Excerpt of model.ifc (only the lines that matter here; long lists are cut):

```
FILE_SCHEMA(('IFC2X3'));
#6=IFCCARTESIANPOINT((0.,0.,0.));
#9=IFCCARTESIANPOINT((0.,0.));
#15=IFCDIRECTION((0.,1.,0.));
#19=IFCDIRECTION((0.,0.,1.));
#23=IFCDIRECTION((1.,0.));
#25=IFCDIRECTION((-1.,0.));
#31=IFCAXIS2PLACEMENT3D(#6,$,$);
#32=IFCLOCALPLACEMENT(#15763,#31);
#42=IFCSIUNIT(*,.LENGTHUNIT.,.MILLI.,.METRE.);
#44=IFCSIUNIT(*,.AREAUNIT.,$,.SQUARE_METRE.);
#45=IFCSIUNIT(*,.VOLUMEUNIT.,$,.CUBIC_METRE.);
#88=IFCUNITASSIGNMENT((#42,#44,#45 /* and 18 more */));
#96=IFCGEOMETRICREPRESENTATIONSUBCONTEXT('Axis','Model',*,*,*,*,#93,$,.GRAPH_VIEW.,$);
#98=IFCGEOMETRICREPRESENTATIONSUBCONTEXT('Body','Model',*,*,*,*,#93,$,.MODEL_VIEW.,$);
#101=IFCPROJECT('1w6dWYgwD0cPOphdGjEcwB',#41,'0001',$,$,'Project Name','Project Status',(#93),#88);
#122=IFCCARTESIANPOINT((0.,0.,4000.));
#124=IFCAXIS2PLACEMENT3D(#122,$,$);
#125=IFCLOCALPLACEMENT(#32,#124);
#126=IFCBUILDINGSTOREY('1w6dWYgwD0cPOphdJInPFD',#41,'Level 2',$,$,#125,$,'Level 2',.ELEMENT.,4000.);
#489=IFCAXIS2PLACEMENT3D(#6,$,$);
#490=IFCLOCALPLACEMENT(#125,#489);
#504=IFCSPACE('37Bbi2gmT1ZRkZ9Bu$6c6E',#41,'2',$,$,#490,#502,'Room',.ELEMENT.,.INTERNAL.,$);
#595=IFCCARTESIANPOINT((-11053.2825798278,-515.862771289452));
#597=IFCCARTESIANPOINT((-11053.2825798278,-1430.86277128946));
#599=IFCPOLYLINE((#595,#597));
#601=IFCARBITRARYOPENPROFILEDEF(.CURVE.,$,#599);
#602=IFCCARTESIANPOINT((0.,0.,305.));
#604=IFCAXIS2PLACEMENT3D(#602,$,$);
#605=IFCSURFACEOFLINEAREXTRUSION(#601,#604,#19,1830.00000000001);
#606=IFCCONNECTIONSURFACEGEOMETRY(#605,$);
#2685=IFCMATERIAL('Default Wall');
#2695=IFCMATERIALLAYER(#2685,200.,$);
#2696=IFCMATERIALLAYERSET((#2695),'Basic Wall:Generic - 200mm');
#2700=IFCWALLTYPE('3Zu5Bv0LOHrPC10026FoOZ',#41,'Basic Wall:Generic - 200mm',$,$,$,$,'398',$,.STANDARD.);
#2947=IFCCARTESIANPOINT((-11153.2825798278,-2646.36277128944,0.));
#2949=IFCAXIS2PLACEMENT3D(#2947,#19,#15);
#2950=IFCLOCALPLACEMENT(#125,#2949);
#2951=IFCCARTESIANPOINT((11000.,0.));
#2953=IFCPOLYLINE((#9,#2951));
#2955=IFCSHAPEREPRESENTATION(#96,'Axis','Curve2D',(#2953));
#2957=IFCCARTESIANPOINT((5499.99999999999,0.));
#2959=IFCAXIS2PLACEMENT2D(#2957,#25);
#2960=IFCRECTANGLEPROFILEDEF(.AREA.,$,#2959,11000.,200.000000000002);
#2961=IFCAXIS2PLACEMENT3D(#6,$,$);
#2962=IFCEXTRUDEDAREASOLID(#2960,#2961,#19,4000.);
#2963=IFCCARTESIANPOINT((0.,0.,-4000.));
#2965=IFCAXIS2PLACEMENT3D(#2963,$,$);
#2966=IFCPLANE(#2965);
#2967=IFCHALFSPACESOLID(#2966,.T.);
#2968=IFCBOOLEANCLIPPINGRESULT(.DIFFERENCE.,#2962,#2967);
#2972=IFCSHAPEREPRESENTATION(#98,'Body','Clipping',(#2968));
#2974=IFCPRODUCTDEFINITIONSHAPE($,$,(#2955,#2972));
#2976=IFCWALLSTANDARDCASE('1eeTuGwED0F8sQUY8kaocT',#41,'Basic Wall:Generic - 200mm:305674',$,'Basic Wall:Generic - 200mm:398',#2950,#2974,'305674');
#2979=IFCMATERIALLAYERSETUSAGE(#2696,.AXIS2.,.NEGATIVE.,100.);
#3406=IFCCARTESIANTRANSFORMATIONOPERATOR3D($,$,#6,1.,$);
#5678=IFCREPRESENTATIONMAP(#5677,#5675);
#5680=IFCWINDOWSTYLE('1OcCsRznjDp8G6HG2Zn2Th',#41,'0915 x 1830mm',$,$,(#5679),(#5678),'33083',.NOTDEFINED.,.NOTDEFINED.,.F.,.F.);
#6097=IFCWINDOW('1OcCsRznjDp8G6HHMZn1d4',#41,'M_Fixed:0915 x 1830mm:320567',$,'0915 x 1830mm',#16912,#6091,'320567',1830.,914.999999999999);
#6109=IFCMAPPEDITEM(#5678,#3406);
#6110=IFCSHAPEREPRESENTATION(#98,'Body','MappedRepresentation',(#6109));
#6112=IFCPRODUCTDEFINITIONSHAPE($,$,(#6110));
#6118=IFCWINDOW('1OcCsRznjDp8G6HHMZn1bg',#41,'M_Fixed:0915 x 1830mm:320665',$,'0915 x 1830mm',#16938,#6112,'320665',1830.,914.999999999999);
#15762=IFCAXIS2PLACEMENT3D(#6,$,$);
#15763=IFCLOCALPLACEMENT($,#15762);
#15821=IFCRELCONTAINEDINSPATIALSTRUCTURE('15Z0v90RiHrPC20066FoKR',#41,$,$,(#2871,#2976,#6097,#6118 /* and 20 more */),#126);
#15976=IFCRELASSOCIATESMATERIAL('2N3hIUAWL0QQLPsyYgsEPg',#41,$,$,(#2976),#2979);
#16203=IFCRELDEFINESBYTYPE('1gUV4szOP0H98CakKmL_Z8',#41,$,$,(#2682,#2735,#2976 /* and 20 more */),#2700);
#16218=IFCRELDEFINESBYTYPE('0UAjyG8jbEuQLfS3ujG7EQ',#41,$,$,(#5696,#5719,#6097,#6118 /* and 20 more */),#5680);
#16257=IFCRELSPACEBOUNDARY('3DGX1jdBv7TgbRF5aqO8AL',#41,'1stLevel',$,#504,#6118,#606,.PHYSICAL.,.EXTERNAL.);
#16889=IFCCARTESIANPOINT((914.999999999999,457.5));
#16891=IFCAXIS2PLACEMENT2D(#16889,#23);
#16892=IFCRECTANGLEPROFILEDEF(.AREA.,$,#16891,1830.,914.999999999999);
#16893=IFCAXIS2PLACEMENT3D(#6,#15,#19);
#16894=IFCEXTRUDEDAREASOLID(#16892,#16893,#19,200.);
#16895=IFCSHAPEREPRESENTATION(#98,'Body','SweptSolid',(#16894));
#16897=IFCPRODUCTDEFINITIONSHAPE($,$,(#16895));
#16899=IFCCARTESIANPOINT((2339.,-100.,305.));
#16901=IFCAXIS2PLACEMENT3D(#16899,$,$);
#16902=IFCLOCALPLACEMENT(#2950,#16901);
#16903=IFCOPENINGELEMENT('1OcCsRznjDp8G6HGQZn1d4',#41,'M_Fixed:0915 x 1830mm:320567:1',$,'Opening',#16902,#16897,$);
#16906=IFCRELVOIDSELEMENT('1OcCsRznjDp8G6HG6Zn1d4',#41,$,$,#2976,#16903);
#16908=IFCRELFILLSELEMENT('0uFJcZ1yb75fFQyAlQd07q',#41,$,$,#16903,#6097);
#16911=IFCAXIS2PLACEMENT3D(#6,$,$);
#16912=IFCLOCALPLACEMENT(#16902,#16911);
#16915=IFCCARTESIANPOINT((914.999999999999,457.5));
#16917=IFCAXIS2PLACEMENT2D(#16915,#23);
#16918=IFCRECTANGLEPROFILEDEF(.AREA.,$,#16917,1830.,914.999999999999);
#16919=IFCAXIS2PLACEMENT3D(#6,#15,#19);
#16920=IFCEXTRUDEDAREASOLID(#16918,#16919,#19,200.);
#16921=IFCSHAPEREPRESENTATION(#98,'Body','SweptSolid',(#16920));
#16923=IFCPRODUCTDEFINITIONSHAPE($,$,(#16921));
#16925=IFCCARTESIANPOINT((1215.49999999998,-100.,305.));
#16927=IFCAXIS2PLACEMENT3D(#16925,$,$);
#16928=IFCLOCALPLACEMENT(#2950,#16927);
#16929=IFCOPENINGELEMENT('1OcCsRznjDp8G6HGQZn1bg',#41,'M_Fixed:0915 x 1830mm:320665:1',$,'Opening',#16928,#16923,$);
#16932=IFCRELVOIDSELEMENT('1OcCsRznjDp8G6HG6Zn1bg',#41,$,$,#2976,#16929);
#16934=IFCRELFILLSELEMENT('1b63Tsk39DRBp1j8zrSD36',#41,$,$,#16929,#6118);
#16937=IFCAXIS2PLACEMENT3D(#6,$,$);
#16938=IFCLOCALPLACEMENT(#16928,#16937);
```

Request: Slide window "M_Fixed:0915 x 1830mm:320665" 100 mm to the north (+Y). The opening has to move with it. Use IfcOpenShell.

```python
import numpy as np
import ifcopenshell
import ifcopenshell.api.geometry
import ifcopenshell.util.placement

model = ifcopenshell.open("model.ifc")

window = model.by_guid("1OcCsRznjDp8G6HHMZn1bg")
opening = window.FillsVoids[0].RelatingOpeningElement
wall = opening.VoidsElements[0].RelatingBuildingElement

wall_matrix = ifcopenshell.util.placement.get_local_placement(wall.ObjectPlacement)
shift = wall_matrix[:3, 0] * 100.0
before = ifcopenshell.util.placement.get_local_placement(window.ObjectPlacement)[:3, 3].copy()

# The window is placed relative to its opening, so it follows when the opening moves.
matrix = ifcopenshell.util.placement.get_local_placement(opening.ObjectPlacement)
matrix[:3, 3] += shift
ifcopenshell.api.geometry.edit_object_placement(
    model, product=opening, matrix=matrix, is_si=False, should_transform_children=True
)

# Space boundary surfaces are stored in each space's coordinates; move them too.
for rel in window.ProvidesBoundaries:
    if not rel.ConnectionGeometry:
        continue
    surface = rel.ConnectionGeometry.SurfaceOnRelatingElement
    space_matrix = ifcopenshell.util.placement.get_local_placement(rel.RelatingSpace.ObjectPlacement)
    point = np.array(surface.Position.Location.Coordinates) + space_matrix[:3, :3].T @ shift
    surface.Position = model.createIfcAxis2Placement3D(
        model.createIfcCartesianPoint(point.tolist()), surface.Position.Axis, surface.Position.RefDirection
    )

after = ifcopenshell.util.placement.get_local_placement(window.ObjectPlacement)[:3, 3]
print("window moved by", (after - before).round(3) + 0.0)

model.write("model_v2.ifc")
```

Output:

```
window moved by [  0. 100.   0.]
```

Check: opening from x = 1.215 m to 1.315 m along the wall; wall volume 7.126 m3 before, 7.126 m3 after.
